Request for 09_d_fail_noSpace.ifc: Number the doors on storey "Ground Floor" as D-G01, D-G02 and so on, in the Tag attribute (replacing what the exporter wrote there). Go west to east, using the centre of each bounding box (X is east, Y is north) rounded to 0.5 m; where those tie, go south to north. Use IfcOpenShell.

First a look at what the model holds.

```python
import ifcopenshell
import ifcopenshell.util.element
import ifcopenshell.util.placement

model = ifcopenshell.open("09_d_fail_noSpace.ifc")
print(model.schema)
storey = next(s for s in model.by_type("IfcBuildingStorey") if s.Name == "Ground Floor")
doors = [e for e in ifcopenshell.util.element.get_decomposition(storey) if e.is_a("IfcDoor")]
for e in sorted(doors, key=lambda e: e.id()):
    origin = ifcopenshell.util.placement.get_local_placement(e.ObjectPlacement)[:3, 3]
    print(e.id(), e.Tag, e.Name, origin.round(2) + 0.0, sep=" | ")
```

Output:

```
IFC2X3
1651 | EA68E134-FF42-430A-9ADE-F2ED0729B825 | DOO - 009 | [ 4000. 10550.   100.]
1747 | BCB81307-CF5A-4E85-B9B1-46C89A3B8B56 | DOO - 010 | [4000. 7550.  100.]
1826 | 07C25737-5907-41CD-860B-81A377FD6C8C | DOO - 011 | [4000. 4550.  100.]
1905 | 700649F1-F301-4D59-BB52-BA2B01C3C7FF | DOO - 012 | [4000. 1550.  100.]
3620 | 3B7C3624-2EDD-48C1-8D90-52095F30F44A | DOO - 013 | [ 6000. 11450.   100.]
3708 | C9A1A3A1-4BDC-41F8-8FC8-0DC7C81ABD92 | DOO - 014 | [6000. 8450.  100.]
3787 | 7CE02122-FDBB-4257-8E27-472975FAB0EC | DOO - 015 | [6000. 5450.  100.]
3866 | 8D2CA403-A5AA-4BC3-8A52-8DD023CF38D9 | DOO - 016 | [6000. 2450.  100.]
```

```python
import ifcopenshell
import ifcopenshell.geom
import ifcopenshell.util.element
import ifcopenshell.util.shape

model = ifcopenshell.open("09_d_fail_noSpace.ifc")
settings = ifcopenshell.geom.settings()
settings.set("use-world-coords", True)


def centre(element):
    shape = ifcopenshell.geom.create_shape(settings, element)
    return ifcopenshell.util.shape.get_bbox_centroid(shape.geometry)


storey = next(s for s in model.by_type("IfcBuildingStorey") if s.Name == "Ground Floor")
doors = [e for e in ifcopenshell.util.element.get_decomposition(storey) if e.is_a("IfcDoor")]

# Insertion points can sit at a corner or the storey origin, so sort by the geometry (in metres).
centres = {e: centre(e) for e in doors}
doors.sort(key=lambda e: (round(centres[e][0] / 0.5), centres[e][1]))

for i, e in enumerate(doors, start=1):
    number = f"D-G{i:02d}"
    e.Tag = number
    print(e.id(), number)

model.write("09_d_fail_noSpace-out.ifc")
```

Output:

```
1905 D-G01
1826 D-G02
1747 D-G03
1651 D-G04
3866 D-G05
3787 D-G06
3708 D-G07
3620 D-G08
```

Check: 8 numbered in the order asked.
